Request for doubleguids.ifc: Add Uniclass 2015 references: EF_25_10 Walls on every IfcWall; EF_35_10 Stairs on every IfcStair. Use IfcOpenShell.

First a look at what the model holds.

```python
import ifcopenshell

model = ifcopenshell.open("doubleguids.ifc")
print(model.schema)
print("classifications:", [c.Name for c in model.by_type("IfcClassification")])
for ifc_class in ("IfcDoor", "IfcRoof", "IfcStair", "IfcWall", "IfcWindow"):
    print(ifc_class, len(model.by_type(ifc_class)))
```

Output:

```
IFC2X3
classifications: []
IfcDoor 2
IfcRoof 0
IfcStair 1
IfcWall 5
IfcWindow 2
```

```python
import ifcopenshell
import ifcopenshell.api.classification

model = ifcopenshell.open("doubleguids.ifc")

# IFC2X3 requires Source and Edition and has no link from the project to the system.
system = model.create_entity("IfcClassification", Source="NBS", Edition="2015", Name="Uniclass 2015")

codes = {
    "IfcWall": ("EF_25_10", "Walls"),
    "IfcStair": ("EF_35_10", "Stairs"),
}
for ifc_class, (code, name) in codes.items():
    products = model.by_type(ifc_class)
    ifcopenshell.api.classification.add_reference(
        model, products=products, classification=system, identification=code, name=name
    )
    print(code, len(products))

model.write("doubleguids_edited.ifc")
```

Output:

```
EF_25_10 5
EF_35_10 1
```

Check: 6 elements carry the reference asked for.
